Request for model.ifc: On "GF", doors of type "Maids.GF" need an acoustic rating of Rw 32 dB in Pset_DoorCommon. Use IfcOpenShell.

First a look at what the model holds.

```python
import ifcopenshell
import ifcopenshell.util.element

model = ifcopenshell.open("model.ifc")
print(model.schema)
storey = next(s for s in model.by_type("IfcBuildingStorey") if s.Name == "GF")
doors = [e for e in ifcopenshell.util.element.get_decomposition(storey) if e.is_a("IfcDoor")]
seen = {}
for e in doors:
    element_type = ifcopenshell.util.element.get_type(e)
    key = (element_type.Name if element_type != e and element_type else None, ifcopenshell.util.element.get_pset(e, "Pset_DoorCommon", "AcousticRating"))
    seen[key] = seen.get(key, 0) + 1
for (name, value), count in sorted(seen.items(), key=str):
    print(count, "x", name, "|", value)
```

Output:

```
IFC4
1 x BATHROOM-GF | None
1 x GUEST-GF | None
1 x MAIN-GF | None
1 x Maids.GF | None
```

```python
import ifcopenshell
import ifcopenshell.api.pset
import ifcopenshell.util.element

model = ifcopenshell.open("model.ifc")

storey = next(s for s in model.by_type("IfcBuildingStorey") if s.Name == "GF")
doors = [e for e in ifcopenshell.util.element.get_decomposition(storey) if e.is_a("IfcDoor")]

count = 0
for e in doors:
    element_type = ifcopenshell.util.element.get_type(e)
    if element_type in (None, e) or element_type.Name != "Maids.GF":
        continue
    # add_pset returns the element's existing set when there is one.
    pset = ifcopenshell.api.pset.add_pset(model, product=e, name="Pset_DoorCommon")
    ifcopenshell.api.pset.edit_pset(model, pset=pset, properties={"AcousticRating": "Rw 32 dB"})
    count += 1

print(count, "doors updated")

model.write("model_updated.ifc")
```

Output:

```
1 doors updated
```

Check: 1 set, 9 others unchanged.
